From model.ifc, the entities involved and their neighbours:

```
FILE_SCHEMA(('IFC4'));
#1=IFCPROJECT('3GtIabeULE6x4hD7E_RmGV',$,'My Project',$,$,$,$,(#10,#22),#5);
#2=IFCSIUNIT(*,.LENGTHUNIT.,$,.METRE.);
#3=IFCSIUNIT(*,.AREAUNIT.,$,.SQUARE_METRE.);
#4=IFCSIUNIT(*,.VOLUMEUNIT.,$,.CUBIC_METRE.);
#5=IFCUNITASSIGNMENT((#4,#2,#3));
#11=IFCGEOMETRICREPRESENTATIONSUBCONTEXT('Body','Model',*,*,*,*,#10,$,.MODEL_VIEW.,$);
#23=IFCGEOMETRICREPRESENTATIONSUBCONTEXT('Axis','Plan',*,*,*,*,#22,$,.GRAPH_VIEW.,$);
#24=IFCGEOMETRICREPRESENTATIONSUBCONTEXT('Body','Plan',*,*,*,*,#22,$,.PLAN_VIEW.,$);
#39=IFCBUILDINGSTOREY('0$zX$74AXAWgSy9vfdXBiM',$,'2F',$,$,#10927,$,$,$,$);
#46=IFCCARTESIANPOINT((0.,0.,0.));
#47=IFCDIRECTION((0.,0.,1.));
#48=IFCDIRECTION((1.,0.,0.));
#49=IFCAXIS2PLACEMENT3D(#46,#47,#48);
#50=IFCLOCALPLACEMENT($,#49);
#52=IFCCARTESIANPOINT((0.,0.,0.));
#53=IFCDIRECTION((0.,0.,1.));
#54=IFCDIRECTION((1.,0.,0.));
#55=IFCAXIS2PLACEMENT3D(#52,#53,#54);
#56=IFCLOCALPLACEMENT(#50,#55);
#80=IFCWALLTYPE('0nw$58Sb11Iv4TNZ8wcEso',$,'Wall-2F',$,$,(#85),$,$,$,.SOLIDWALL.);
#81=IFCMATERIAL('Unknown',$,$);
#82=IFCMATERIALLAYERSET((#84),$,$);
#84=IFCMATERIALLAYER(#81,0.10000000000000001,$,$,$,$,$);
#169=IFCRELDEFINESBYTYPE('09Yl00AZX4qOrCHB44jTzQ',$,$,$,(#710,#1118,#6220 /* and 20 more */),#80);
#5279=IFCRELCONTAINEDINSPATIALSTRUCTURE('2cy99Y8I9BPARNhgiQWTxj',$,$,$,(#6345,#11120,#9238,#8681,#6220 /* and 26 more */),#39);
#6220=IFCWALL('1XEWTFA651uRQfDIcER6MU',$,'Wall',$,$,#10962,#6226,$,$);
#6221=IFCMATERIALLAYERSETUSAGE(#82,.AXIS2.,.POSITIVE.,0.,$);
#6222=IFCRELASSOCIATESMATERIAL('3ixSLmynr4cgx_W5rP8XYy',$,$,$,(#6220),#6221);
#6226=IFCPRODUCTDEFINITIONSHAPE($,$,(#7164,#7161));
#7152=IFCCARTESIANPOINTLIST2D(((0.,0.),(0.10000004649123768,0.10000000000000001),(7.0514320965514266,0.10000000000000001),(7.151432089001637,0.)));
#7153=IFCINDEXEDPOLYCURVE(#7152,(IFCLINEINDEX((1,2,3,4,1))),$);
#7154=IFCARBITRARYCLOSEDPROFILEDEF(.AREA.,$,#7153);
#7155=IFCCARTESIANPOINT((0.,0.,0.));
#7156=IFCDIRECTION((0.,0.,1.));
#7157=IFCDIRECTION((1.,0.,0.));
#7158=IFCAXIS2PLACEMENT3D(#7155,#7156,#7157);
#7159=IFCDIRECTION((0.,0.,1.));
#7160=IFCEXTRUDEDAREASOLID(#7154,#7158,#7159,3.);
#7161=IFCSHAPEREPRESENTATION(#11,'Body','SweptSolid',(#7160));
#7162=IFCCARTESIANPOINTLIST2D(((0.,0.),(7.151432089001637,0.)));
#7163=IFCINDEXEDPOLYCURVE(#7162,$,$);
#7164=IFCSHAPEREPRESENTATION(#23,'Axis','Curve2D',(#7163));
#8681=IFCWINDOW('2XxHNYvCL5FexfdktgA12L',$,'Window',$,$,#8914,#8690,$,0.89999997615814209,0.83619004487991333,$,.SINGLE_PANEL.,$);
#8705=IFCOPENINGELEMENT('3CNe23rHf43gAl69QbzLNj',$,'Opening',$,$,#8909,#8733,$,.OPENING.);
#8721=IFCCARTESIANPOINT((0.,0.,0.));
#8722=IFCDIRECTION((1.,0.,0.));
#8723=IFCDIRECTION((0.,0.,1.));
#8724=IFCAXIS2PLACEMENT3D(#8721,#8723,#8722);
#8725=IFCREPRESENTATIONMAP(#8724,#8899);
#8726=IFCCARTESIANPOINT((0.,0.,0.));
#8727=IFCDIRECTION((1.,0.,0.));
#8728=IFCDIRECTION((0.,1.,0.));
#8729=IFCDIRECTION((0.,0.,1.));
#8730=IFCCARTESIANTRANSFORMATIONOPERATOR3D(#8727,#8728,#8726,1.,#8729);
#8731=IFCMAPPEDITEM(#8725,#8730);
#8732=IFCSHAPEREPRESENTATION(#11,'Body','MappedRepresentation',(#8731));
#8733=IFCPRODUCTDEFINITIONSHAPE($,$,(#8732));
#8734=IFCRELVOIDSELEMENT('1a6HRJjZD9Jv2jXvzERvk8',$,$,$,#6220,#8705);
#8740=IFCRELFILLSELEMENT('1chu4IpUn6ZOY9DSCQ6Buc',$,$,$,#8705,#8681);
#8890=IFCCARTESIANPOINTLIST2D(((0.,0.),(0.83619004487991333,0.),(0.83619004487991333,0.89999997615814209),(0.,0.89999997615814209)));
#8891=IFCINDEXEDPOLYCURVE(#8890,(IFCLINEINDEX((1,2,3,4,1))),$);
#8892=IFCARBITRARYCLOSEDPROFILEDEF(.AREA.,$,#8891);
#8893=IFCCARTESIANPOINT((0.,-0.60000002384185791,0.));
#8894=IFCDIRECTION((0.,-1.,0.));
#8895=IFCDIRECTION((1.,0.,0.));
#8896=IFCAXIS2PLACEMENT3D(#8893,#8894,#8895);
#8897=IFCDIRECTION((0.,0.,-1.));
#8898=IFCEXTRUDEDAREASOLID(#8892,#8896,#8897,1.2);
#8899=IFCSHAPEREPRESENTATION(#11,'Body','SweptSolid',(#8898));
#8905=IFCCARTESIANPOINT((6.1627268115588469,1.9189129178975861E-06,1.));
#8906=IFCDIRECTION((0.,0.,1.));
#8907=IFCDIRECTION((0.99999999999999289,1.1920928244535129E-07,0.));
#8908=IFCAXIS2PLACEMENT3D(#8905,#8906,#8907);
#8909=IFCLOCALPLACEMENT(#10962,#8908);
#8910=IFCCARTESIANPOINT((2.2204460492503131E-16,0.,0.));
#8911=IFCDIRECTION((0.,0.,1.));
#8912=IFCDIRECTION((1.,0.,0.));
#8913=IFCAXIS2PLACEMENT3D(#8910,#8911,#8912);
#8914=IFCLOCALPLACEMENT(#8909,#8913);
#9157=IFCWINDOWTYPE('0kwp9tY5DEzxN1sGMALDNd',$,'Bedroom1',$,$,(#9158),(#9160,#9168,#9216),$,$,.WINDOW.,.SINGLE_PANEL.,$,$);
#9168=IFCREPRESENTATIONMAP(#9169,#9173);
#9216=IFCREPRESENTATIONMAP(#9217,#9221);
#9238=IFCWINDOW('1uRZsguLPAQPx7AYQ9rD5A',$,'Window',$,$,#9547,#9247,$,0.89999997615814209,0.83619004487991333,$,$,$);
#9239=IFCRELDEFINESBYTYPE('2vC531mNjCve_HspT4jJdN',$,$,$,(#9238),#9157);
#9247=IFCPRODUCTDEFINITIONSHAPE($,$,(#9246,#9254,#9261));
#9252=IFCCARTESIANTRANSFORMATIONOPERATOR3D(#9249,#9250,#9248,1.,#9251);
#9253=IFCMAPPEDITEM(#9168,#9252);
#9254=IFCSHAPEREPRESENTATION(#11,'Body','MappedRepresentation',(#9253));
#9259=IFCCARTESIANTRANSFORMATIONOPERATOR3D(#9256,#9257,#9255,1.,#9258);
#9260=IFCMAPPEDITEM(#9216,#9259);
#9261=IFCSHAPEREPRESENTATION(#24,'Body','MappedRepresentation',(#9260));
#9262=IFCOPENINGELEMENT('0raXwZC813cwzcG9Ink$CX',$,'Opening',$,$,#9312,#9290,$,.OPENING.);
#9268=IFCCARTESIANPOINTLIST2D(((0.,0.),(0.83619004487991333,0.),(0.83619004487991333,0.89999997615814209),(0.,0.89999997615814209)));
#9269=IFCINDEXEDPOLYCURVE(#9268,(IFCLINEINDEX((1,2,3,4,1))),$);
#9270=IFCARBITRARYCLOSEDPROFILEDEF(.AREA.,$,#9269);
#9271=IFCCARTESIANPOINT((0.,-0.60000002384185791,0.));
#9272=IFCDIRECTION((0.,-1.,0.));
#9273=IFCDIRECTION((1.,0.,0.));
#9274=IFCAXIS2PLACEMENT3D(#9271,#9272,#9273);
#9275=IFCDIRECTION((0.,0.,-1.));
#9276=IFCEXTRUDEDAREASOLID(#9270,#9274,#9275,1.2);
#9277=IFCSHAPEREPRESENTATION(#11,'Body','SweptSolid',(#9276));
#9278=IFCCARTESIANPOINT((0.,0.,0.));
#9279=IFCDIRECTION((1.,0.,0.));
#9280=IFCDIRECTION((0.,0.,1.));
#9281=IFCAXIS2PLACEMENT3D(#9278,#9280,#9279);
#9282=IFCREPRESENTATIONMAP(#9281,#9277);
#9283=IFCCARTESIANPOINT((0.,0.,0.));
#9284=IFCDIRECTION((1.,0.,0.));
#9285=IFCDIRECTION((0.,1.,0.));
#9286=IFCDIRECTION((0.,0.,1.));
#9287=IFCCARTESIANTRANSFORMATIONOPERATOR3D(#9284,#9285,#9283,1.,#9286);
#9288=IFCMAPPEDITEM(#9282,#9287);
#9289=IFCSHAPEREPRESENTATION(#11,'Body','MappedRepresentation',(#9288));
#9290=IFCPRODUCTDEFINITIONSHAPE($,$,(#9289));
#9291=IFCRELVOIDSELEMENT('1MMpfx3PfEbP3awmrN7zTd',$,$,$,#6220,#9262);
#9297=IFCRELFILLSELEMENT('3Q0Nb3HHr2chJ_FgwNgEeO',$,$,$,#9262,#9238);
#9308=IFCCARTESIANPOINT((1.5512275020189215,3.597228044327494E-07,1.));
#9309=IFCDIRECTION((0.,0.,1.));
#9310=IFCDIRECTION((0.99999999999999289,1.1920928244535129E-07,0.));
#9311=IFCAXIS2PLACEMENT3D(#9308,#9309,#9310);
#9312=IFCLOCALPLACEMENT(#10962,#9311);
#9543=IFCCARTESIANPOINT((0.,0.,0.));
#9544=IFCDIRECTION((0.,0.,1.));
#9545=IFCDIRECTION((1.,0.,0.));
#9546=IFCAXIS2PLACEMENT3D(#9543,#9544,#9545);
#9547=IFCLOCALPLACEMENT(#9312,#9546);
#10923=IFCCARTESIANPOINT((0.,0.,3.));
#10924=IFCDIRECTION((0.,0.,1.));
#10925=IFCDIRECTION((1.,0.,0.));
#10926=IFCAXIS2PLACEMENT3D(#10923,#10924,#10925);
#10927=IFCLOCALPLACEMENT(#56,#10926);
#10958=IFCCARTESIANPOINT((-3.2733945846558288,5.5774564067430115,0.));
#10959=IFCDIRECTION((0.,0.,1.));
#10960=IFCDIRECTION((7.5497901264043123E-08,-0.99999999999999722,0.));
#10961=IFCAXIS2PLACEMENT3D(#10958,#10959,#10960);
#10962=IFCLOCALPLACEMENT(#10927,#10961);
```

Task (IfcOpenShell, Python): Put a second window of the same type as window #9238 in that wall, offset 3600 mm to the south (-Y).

```python
import ifcopenshell
import ifcopenshell.api.feature
import ifcopenshell.api.geometry
import ifcopenshell.api.root
import ifcopenshell.geom
import ifcopenshell.util.element
import ifcopenshell.util.placement
import ifcopenshell.util.shape

model = ifcopenshell.open("model.ifc")
settings = ifcopenshell.geom.settings()


def volume(element):
    """Net volume in cubic metres, openings subtracted."""
    shape = ifcopenshell.geom.create_shape(settings, element)
    return ifcopenshell.util.shape.get_volume(shape.geometry)


window = model.by_guid("1uRZsguLPAQPx7AYQ9rD5A")
opening = window.FillsVoids[0].RelatingOpeningElement
wall = opening.VoidsElements[0].RelatingBuildingElement
before = volume(wall)
shift = ifcopenshell.util.placement.get_local_placement(wall.ObjectPlacement)[:3, 0] * 3.6

# copy_class copies the void relationship, type, container and properties, but no geometry.
new_opening = ifcopenshell.api.root.copy_class(model, product=opening)
new_opening.Representation = ifcopenshell.util.element.copy_deep(
    model, opening.Representation, exclude=["IfcGeometricRepresentationContext", "IfcRepresentationMap"]
)
new_window = ifcopenshell.api.root.copy_class(model, product=window)
new_window.Representation = ifcopenshell.util.element.copy_deep(
    model, window.Representation, exclude=["IfcGeometricRepresentationContext", "IfcRepresentationMap"]
)
ifcopenshell.api.feature.add_filling(model, opening=new_opening, element=new_window)

for old, new in ((opening, new_opening), (window, new_window)):
    matrix = ifcopenshell.util.placement.get_local_placement(old.ObjectPlacement)
    matrix[:3, 3] += shift
    ifcopenshell.api.geometry.edit_object_placement(model, product=new, matrix=matrix, is_si=False)

after = volume(wall)

print(f"wall volume {before:.3f} -> {after:.3f} m3")

model.write("model-out.ifc")
```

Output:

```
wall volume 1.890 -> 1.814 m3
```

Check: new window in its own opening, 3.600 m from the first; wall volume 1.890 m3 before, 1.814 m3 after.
